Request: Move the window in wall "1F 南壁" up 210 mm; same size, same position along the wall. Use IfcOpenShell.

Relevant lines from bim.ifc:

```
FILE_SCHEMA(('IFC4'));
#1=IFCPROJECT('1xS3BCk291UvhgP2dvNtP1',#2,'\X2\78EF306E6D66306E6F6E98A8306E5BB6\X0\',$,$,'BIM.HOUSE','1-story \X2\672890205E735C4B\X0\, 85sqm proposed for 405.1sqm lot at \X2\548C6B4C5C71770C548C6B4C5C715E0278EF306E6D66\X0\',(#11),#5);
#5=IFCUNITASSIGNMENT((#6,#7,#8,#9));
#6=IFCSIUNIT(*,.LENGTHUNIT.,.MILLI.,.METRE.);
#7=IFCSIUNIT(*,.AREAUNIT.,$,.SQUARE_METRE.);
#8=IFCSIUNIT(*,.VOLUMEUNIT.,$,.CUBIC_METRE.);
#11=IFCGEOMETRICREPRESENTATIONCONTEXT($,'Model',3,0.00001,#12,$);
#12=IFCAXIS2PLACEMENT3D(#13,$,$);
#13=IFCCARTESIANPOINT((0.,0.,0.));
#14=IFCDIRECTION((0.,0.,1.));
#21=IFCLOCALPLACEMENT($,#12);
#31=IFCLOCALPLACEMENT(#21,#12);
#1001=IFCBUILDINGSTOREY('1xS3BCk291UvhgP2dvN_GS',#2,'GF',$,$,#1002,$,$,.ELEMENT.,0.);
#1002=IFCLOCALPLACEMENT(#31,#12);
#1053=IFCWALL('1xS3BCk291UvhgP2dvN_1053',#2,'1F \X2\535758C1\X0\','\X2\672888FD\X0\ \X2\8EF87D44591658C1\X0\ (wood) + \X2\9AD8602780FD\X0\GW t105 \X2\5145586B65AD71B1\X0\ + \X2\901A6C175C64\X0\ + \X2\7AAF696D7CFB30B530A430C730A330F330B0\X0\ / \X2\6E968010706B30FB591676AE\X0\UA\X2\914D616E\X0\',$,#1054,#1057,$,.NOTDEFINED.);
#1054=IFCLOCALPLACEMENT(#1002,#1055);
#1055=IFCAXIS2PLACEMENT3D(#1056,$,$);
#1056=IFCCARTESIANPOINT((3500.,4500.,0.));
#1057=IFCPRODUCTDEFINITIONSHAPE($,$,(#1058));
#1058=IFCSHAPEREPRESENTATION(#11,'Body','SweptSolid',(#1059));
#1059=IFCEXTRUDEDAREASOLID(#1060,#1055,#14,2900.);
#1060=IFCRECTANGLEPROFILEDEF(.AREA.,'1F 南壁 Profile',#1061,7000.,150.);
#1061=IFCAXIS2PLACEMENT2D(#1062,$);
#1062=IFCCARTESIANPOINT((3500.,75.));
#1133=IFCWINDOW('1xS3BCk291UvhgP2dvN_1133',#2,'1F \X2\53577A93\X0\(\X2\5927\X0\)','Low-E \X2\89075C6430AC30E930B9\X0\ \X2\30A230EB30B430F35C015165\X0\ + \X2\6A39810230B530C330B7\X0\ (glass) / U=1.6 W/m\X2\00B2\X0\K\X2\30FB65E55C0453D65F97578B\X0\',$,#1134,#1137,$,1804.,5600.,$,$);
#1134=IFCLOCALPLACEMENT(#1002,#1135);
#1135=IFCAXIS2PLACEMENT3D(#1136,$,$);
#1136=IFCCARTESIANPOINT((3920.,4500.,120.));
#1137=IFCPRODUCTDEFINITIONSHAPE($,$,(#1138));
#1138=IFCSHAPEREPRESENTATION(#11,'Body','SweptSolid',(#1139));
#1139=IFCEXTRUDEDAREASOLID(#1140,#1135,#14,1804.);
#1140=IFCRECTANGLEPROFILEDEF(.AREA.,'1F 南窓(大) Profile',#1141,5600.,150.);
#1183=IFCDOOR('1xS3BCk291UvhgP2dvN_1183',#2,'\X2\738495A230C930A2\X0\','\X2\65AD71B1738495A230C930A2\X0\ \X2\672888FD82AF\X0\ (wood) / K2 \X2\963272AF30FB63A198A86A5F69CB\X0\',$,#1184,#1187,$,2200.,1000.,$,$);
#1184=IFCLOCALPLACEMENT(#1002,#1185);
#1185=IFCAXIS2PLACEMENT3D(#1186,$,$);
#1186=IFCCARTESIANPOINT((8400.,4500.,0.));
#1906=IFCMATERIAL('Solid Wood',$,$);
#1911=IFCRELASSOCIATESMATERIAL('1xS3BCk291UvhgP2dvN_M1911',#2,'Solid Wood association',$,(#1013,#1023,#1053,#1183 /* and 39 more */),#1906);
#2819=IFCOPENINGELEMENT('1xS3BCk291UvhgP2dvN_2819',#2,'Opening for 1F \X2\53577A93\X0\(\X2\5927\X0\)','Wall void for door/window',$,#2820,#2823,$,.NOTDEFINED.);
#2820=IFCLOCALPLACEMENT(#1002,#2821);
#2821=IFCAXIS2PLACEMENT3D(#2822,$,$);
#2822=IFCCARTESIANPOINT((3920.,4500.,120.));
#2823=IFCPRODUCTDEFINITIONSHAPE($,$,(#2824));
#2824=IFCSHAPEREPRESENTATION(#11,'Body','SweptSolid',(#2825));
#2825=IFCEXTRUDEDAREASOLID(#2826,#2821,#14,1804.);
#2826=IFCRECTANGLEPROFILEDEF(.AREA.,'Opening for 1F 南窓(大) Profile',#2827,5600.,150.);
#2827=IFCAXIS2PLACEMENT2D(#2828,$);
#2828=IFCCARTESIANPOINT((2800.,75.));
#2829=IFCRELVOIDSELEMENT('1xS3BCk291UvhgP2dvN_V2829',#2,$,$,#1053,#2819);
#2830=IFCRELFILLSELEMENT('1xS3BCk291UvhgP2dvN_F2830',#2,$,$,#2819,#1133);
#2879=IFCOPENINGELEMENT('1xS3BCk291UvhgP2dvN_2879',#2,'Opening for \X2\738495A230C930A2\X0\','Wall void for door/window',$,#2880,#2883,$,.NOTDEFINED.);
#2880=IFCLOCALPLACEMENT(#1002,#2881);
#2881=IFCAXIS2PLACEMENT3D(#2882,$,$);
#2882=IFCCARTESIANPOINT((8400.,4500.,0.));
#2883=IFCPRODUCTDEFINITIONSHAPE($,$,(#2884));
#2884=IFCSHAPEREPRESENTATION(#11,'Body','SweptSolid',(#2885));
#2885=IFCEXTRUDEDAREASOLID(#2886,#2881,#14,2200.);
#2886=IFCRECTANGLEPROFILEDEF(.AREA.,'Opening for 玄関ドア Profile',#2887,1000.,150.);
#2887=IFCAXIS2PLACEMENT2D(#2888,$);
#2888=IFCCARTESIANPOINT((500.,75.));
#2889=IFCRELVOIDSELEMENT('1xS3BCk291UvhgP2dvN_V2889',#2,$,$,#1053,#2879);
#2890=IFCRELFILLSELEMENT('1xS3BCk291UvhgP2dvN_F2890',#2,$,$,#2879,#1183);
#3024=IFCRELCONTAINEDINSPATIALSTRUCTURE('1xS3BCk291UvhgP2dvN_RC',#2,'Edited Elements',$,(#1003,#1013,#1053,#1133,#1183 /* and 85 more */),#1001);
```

```python
import numpy as np
import ifcopenshell
import ifcopenshell.api.geometry
import ifcopenshell.util.placement
import ifcopenshell.util.unit

model = ifcopenshell.open("bim.ifc")
unit_scale = ifcopenshell.util.unit.calculate_unit_scale(model)

window = model.by_guid("1xS3BCk291UvhgP2dvN_1133")
opening = window.FillsVoids[0].RelatingOpeningElement
dz = 210.0

shift = np.array([0.0, 0.0, dz])
# The window is not placed relative to its opening, so move both.
for product in (opening, window):
    matrix = ifcopenshell.util.placement.get_local_placement(product.ObjectPlacement)
    matrix[:3, 3] += shift
    ifcopenshell.api.geometry.edit_object_placement(model, product=product, matrix=matrix, is_si=False)

print(f"moved by {dz * unit_scale:+.3f} m")

model.write("bim_edited.ifc")
```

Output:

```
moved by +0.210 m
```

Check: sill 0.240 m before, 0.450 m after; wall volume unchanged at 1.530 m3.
